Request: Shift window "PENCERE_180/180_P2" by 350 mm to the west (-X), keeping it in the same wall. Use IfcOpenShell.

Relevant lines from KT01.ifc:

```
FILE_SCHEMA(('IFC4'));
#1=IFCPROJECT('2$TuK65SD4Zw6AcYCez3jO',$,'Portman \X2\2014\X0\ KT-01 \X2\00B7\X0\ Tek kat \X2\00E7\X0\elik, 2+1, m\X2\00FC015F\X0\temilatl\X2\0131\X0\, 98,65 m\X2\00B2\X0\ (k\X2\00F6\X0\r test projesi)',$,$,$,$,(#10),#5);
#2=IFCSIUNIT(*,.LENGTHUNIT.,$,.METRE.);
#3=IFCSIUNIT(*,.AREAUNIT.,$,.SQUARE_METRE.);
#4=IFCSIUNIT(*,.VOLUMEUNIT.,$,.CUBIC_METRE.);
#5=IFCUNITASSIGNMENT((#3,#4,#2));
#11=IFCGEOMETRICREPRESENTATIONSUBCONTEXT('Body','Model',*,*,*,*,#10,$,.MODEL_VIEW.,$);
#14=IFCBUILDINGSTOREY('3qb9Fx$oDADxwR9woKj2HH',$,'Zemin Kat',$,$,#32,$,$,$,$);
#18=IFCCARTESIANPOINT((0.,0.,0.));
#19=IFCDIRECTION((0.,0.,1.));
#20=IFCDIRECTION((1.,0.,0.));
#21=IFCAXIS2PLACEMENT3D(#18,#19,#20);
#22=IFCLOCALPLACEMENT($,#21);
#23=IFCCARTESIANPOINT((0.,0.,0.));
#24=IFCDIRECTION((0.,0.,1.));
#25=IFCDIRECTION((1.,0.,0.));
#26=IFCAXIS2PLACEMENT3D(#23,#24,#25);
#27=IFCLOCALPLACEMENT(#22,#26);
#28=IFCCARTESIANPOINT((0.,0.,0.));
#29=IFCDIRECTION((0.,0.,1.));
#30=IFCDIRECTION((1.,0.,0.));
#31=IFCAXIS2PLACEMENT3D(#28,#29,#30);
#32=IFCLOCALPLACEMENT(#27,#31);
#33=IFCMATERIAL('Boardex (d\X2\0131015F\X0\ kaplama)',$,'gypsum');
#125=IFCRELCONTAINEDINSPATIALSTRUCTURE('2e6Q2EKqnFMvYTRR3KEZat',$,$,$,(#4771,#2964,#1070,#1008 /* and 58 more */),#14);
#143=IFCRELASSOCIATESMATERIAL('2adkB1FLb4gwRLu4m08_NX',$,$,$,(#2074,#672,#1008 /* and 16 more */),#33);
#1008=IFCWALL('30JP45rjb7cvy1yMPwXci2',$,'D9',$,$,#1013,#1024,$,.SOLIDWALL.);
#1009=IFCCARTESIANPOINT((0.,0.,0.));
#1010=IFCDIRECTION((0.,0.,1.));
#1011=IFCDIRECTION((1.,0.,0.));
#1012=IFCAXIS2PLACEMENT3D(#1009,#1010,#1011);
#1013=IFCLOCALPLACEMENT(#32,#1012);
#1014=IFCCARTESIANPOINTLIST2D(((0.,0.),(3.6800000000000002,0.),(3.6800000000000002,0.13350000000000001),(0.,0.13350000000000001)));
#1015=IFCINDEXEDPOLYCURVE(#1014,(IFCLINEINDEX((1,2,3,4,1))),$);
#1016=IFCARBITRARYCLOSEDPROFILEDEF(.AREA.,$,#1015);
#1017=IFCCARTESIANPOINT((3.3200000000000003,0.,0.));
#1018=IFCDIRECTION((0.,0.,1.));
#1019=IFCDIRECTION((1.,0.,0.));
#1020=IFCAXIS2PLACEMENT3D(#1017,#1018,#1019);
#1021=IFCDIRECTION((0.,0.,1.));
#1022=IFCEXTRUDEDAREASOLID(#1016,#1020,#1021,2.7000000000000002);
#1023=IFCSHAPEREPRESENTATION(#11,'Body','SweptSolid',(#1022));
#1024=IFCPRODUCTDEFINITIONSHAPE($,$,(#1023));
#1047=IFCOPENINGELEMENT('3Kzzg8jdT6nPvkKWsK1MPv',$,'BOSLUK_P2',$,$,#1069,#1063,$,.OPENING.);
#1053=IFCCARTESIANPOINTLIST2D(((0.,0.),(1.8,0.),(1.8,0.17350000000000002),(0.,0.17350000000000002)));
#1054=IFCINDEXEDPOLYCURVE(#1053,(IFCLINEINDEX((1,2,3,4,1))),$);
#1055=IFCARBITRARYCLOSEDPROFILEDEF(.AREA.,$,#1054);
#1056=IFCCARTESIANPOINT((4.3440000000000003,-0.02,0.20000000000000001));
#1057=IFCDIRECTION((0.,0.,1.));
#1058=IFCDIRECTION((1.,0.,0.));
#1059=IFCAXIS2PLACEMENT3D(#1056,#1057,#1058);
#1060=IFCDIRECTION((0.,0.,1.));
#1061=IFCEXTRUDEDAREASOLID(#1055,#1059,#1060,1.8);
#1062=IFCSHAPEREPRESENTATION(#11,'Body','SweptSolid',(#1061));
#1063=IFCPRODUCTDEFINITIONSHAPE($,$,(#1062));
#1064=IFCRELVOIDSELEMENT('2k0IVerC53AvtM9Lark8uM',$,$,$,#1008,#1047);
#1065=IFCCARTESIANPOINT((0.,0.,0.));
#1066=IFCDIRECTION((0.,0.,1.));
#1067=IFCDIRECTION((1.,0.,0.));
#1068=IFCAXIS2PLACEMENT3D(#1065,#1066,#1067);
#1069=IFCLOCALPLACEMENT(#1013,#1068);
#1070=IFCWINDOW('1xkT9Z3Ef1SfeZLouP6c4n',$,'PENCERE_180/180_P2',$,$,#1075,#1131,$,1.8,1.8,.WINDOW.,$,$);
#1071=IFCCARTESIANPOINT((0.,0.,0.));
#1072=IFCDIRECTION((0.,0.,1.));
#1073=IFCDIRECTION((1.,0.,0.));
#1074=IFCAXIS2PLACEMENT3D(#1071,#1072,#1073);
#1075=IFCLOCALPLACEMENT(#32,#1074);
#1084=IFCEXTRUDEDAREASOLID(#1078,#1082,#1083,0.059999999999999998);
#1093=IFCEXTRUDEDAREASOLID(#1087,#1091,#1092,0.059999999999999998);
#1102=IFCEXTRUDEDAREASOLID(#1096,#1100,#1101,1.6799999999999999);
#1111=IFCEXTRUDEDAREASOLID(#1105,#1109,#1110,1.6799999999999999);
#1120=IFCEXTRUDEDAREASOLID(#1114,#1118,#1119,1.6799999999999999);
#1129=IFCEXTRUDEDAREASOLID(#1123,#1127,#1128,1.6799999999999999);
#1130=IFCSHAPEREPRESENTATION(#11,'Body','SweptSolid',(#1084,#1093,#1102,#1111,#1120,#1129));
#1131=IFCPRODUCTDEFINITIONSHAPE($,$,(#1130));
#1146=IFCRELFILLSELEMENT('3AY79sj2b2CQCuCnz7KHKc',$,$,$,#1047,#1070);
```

```python
import ifcopenshell
import ifcopenshell.api.geometry
import ifcopenshell.util.placement
import ifcopenshell.util.unit

model = ifcopenshell.open("KT01.ifc")
unit_scale = ifcopenshell.util.unit.calculate_unit_scale(model)

window = model.by_guid("1xkT9Z3Ef1SfeZLouP6c4n")
opening = window.FillsVoids[0].RelatingOpeningElement
wall = opening.VoidsElements[0].RelatingBuildingElement

wall_matrix = ifcopenshell.util.placement.get_local_placement(wall.ObjectPlacement)
shift = wall_matrix[:3, 0] * -0.35 / unit_scale
before = ifcopenshell.util.placement.get_local_placement(window.ObjectPlacement)[:3, 3].copy()

# The window is not placed relative to its opening, so move both.
for product in (opening, window):
    matrix = ifcopenshell.util.placement.get_local_placement(product.ObjectPlacement)
    matrix[:3, 3] += shift
    ifcopenshell.api.geometry.edit_object_placement(model, product=product, matrix=matrix, is_si=False)

after = ifcopenshell.util.placement.get_local_placement(window.ObjectPlacement)[:3, 3]
print("window moved by", (after - before).round(3) + 0.0)

model.write("KT01_v2.ifc")
```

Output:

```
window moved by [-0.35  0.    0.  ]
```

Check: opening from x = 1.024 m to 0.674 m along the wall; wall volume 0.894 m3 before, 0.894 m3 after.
